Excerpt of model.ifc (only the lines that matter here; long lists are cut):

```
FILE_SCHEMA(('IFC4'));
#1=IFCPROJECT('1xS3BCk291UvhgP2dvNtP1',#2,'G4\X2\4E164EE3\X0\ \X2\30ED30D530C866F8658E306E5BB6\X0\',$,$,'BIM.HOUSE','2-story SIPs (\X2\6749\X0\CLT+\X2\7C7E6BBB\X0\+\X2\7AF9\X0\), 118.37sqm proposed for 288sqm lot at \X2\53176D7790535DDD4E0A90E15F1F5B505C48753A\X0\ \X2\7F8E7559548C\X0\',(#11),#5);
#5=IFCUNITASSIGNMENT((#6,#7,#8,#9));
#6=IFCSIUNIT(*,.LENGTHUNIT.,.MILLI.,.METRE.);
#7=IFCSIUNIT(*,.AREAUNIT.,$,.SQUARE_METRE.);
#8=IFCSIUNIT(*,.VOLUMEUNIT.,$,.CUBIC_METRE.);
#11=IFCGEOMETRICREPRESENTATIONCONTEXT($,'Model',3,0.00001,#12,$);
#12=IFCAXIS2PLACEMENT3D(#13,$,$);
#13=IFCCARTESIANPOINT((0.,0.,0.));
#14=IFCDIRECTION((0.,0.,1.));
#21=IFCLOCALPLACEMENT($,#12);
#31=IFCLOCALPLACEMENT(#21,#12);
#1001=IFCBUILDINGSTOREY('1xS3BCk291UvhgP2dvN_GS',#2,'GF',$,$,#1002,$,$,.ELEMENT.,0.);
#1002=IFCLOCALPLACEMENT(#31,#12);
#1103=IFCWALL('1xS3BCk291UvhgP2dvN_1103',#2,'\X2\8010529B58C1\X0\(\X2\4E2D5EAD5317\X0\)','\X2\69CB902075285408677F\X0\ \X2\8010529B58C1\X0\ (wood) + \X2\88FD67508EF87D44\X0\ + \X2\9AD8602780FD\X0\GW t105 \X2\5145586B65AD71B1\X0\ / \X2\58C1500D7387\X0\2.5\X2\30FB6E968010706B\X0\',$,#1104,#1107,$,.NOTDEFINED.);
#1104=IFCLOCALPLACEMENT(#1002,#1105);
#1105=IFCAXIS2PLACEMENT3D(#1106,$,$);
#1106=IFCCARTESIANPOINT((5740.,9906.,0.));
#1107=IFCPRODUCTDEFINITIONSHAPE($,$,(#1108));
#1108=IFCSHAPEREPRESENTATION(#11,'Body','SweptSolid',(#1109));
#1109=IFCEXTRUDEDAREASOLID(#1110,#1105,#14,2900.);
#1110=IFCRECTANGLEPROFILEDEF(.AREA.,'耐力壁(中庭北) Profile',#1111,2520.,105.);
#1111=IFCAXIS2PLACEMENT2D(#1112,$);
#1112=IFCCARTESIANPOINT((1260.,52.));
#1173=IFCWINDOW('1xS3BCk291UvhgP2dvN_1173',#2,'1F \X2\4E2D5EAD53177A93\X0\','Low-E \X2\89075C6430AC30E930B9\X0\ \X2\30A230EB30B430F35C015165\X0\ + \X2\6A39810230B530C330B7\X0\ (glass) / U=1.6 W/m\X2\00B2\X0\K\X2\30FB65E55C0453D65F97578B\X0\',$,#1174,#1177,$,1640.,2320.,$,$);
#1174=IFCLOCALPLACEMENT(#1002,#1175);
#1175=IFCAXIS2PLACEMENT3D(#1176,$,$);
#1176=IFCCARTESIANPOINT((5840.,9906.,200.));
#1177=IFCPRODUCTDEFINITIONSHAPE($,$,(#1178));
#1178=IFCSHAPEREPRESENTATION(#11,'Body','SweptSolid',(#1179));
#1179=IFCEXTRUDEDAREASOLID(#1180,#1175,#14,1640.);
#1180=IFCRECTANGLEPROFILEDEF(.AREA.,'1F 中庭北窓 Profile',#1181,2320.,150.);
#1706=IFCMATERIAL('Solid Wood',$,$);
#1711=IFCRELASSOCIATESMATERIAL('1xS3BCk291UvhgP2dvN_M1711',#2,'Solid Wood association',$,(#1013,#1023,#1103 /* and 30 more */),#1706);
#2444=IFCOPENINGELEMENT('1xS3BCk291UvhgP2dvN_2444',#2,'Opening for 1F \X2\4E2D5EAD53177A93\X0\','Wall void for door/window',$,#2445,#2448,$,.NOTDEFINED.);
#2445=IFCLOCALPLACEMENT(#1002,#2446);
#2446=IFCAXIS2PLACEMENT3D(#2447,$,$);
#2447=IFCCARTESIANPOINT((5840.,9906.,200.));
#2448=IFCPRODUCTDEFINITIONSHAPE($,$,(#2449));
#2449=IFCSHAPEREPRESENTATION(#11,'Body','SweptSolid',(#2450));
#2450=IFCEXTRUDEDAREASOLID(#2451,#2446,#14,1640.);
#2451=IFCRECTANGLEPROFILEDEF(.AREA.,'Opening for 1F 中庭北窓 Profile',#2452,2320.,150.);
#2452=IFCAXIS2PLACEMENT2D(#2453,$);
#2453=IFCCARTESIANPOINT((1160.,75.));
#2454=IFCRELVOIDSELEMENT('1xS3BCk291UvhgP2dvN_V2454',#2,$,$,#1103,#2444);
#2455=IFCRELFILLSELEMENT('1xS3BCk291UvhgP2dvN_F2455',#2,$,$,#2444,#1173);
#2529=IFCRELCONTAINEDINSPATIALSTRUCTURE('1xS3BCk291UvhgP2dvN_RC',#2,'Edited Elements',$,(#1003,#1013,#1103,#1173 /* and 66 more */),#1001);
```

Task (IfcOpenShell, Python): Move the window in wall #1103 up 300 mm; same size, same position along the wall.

```python
import numpy as np
import ifcopenshell
import ifcopenshell.api.geometry
import ifcopenshell.util.placement
import ifcopenshell.util.unit

model = ifcopenshell.open("model.ifc")
unit_scale = ifcopenshell.util.unit.calculate_unit_scale(model)

window = model.by_id(1173)
opening = window.FillsVoids[0].RelatingOpeningElement
dz = 300.0

shift = np.array([0.0, 0.0, dz])
# The window is not placed relative to its opening, so move both.
for product in (opening, window):
    matrix = ifcopenshell.util.placement.get_local_placement(product.ObjectPlacement)
    matrix[:3, 3] += shift
    ifcopenshell.api.geometry.edit_object_placement(model, product=product, matrix=matrix, is_si=False)

print(f"moved by {dz * unit_scale:+.3f} m")

model.write("model_edited.ifc")
```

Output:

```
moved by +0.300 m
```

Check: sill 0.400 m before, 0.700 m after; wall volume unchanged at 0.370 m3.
